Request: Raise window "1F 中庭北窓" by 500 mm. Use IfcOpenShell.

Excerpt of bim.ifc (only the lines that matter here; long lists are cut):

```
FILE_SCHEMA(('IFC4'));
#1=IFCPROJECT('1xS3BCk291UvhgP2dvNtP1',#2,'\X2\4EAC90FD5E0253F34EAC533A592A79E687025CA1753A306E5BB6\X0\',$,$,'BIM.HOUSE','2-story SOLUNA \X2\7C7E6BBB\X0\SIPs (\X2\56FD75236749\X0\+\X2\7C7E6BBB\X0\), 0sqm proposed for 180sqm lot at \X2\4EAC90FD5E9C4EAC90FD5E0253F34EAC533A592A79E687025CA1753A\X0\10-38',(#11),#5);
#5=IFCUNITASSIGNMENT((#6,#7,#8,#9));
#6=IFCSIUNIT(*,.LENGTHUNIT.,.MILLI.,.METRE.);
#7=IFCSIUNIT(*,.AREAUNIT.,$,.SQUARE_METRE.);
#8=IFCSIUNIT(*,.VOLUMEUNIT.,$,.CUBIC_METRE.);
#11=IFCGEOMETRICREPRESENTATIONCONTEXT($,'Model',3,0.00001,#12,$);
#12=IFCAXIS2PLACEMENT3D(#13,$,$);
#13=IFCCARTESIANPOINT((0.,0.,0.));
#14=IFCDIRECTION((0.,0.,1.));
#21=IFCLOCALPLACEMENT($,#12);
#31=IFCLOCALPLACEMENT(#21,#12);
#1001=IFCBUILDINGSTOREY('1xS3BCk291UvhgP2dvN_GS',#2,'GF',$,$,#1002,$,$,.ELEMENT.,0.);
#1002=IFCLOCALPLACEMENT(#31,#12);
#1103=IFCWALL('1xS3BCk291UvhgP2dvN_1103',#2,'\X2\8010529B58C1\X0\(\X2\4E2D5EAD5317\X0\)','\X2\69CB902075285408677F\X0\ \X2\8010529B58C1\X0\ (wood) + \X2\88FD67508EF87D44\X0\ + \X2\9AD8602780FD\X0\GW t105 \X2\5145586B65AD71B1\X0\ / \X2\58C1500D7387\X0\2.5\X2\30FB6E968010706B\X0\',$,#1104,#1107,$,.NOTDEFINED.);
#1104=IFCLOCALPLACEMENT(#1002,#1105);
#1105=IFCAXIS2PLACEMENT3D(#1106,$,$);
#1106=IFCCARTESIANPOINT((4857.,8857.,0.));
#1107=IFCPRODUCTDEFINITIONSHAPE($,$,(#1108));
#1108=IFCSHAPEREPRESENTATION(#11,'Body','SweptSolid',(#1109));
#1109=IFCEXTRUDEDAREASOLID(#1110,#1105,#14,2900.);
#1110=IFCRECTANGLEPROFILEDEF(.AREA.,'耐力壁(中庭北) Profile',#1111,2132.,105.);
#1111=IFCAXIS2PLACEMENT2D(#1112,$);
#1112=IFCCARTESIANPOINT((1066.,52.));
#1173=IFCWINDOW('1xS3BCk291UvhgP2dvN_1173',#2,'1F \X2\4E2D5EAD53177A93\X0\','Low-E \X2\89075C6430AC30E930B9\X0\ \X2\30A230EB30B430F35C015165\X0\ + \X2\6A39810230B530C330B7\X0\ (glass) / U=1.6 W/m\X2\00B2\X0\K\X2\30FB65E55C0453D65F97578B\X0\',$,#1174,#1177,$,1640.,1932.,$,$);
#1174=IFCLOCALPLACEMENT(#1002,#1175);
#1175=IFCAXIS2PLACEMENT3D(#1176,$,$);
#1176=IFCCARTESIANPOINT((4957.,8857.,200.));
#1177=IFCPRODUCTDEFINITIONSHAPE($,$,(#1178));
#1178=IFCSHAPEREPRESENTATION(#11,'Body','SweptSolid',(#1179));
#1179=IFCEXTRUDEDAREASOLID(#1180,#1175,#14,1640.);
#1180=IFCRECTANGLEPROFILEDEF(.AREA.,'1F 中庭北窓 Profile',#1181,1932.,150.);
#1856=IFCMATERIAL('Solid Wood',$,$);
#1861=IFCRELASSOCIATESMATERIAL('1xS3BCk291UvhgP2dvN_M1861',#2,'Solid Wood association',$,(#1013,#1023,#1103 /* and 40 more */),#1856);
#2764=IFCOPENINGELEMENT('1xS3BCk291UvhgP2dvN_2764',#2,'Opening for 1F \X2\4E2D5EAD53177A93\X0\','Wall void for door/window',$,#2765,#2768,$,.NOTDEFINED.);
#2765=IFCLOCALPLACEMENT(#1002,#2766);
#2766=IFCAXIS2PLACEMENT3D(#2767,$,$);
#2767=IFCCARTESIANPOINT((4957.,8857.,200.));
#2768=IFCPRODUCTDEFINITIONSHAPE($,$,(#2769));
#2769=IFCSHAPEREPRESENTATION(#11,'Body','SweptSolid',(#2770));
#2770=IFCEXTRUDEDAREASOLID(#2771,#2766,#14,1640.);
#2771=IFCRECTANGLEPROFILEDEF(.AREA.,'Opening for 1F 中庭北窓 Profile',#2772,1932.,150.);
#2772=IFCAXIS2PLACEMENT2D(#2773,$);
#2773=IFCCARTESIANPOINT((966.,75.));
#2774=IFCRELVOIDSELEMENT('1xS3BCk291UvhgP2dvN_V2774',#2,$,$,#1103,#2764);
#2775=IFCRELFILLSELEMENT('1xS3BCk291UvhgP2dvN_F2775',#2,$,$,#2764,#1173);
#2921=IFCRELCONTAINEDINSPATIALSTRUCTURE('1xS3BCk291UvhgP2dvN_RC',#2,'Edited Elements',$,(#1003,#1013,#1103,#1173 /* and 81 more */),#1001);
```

```python
import numpy as np
import ifcopenshell
import ifcopenshell.api.geometry
import ifcopenshell.util.placement
import ifcopenshell.util.unit

model = ifcopenshell.open("bim.ifc")
unit_scale = ifcopenshell.util.unit.calculate_unit_scale(model)

window = model.by_id(1173)
opening = window.FillsVoids[0].RelatingOpeningElement
dz = 500.0

shift = np.array([0.0, 0.0, dz])
# The window is not placed relative to its opening, so move both.
for product in (opening, window):
    matrix = ifcopenshell.util.placement.get_local_placement(product.ObjectPlacement)
    matrix[:3, 3] += shift
    ifcopenshell.api.geometry.edit_object_placement(model, product=product, matrix=matrix, is_si=False)

print(f"moved by {dz * unit_scale:+.3f} m")

model.write("bim_v2.ifc")
```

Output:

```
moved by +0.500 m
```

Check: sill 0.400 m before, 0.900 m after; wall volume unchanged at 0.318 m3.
